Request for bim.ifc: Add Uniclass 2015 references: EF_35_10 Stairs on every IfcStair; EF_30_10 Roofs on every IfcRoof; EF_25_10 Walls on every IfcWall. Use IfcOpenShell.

First a look at what the model holds.

```python
import ifcopenshell

model = ifcopenshell.open("bim.ifc")
print(model.schema)
print("classifications:", [c.Name for c in model.by_type("IfcClassification")])
for ifc_class in ("IfcDoor", "IfcRoof", "IfcStair", "IfcWall", "IfcWindow"):
    print(ifc_class, len(model.by_type(ifc_class)))
```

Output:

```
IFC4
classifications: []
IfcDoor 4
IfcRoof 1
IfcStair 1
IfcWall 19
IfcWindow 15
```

```python
import ifcopenshell
import ifcopenshell.api.classification

model = ifcopenshell.open("bim.ifc")

system = ifcopenshell.api.classification.add_classification(model, classification="Uniclass 2015")

codes = {
    "IfcStair": ("EF_35_10", "Stairs"),
    "IfcRoof": ("EF_30_10", "Roofs"),
    "IfcWall": ("EF_25_10", "Walls"),
}
for ifc_class, (code, name) in codes.items():
    products = model.by_type(ifc_class)
    ifcopenshell.api.classification.add_reference(
        model, products=products, classification=system, identification=code, name=name
    )
    print(code, len(products))

model.write("bim_rev.ifc")
```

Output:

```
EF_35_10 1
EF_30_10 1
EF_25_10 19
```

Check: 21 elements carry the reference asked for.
